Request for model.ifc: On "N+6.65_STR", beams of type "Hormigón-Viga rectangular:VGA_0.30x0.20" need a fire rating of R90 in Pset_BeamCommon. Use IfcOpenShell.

First a look at what the model holds.

```python
import ifcopenshell
import ifcopenshell.util.element

model = ifcopenshell.open("model.ifc")
print(model.schema)
storey = next(s for s in model.by_type("IfcBuildingStorey") if s.Name == "N+6.65_STR")
beams = [e for e in ifcopenshell.util.element.get_decomposition(storey) if e.is_a("IfcBeam")]
seen = {}
for e in beams:
    element_type = ifcopenshell.util.element.get_type(e)
    key = (element_type.Name if element_type != e and element_type else None, ifcopenshell.util.element.get_pset(e, "Pset_BeamCommon", "FireRating"))
    seen[key] = seen.get(key, 0) + 1
for (name, value), count in sorted(seen.items(), key=str):
    print(count, "x", name, "|", value)
```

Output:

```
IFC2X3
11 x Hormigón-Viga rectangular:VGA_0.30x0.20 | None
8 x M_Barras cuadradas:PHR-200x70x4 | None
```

```python
import ifcopenshell
import ifcopenshell.api.pset
import ifcopenshell.util.element

model = ifcopenshell.open("model.ifc")

storey = next(s for s in model.by_type("IfcBuildingStorey") if s.Name == "N+6.65_STR")
beams = [e for e in ifcopenshell.util.element.get_decomposition(storey) if e.is_a("IfcBeam")]

count = 0
for e in beams:
    element_type = ifcopenshell.util.element.get_type(e)
    if element_type in (None, e) or element_type.Name != "Hormigón-Viga rectangular:VGA_0.30x0.20":
        continue
    # add_pset returns the element's existing set when there is one.
    pset = ifcopenshell.api.pset.add_pset(model, product=e, name="Pset_BeamCommon")
    ifcopenshell.api.pset.edit_pset(model, pset=pset, properties={"FireRating": "R90"})
    count += 1

print(count, "beams updated")

model.write("model_updated.ifc")
```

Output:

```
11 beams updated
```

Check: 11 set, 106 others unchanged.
